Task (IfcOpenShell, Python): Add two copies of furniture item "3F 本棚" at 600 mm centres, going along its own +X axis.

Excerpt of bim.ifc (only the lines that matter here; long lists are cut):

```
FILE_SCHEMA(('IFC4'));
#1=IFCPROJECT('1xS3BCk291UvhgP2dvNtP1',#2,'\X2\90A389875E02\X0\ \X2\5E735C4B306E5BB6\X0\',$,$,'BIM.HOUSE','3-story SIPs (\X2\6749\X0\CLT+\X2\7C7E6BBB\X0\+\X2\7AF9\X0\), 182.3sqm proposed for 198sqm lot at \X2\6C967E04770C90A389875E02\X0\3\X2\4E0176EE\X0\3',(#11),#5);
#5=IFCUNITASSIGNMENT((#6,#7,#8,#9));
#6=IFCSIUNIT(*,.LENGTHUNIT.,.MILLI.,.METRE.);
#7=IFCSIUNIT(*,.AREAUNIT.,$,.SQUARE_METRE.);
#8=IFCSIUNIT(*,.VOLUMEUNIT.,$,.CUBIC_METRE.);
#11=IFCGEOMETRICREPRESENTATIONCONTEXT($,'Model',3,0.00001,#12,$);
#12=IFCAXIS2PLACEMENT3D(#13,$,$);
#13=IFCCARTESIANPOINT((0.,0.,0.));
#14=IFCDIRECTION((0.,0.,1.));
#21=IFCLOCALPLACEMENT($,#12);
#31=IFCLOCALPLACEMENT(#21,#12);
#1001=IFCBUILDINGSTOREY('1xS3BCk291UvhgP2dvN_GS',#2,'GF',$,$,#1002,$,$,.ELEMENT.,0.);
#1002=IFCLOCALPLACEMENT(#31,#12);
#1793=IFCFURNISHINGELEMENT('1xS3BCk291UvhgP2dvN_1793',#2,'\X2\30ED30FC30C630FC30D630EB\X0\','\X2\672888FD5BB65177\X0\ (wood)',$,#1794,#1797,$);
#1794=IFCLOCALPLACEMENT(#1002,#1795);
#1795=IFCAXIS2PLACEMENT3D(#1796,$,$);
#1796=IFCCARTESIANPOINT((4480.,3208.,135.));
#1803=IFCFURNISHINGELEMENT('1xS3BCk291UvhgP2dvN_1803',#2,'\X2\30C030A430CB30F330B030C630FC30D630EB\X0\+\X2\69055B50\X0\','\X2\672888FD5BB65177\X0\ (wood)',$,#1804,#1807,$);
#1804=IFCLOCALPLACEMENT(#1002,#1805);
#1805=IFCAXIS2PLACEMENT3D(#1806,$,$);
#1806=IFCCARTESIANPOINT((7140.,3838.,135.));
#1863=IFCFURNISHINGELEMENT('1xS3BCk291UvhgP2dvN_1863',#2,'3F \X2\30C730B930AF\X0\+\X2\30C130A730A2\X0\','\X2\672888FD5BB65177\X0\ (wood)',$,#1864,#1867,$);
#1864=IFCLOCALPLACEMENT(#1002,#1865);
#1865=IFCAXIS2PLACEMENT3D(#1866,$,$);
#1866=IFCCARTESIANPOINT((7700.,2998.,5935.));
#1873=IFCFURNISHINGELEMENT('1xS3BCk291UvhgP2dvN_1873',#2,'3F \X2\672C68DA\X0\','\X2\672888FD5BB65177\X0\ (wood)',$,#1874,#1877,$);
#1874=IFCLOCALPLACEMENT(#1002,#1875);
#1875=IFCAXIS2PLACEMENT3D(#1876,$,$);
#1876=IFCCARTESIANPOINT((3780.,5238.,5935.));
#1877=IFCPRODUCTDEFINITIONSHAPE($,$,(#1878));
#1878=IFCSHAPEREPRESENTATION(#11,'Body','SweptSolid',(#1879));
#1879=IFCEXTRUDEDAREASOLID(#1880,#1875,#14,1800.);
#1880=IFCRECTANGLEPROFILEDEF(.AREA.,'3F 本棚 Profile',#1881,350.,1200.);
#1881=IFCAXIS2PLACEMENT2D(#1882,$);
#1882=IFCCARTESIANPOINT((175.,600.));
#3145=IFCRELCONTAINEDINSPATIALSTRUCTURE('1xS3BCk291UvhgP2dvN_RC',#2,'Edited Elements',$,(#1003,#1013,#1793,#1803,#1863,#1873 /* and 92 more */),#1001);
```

```python
import ifcopenshell
import ifcopenshell.api.geometry
import ifcopenshell.api.root
import ifcopenshell.util.element
import ifcopenshell.util.placement
import ifcopenshell.util.unit

model = ifcopenshell.open("bim.ifc")
unit_scale = ifcopenshell.util.unit.calculate_unit_scale(model)


def reuse_history(source, copy):
    """copy_class also copies each property set's owner history, people and application; keep the originals."""
    for rel in copy.IsDefinedBy:
        if rel.is_a("IfcRelDefinesByProperties") and (history := rel.RelatingPropertyDefinition.OwnerHistory):
            rel.RelatingPropertyDefinition.OwnerHistory = source.OwnerHistory
            ifcopenshell.util.element.remove_deep2(model, history)


source = model.by_guid("1xS3BCk291UvhgP2dvN_1873")
base = ifcopenshell.util.placement.get_local_placement(source.ObjectPlacement)
step = base[:3, 0] * 0.6 / unit_scale

for i in range(1, 3):
    copy = ifcopenshell.api.root.copy_class(model, product=source)
    copy.Representation = ifcopenshell.util.element.copy_deep(
        model, source.Representation, exclude=["IfcGeometricRepresentationContext", "IfcRepresentationMap"]
    )
    reuse_history(source, copy)
    matrix = base.copy()
    matrix[:3, 3] += i * step
    print("added at", matrix[:3, 3].round(3) + 0.0)
    ifcopenshell.api.geometry.edit_object_placement(model, product=copy, matrix=matrix, is_si=False)

model.write("bim_rev.ifc")
```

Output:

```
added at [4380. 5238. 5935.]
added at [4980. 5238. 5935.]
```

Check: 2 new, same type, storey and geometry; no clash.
